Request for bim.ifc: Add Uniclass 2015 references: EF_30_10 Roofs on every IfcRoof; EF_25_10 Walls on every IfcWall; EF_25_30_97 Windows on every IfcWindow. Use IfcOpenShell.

First a look at what the model holds.

```python
import ifcopenshell

model = ifcopenshell.open("bim.ifc")
print(model.schema)
print("classifications:", [c.Name for c in model.by_type("IfcClassification")])
for ifc_class in ("IfcDoor", "IfcRoof", "IfcStair", "IfcWall", "IfcWindow"):
    print(ifc_class, len(model.by_type(ifc_class)))
```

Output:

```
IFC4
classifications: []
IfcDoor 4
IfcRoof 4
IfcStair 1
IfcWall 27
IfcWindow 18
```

```python
import ifcopenshell
import ifcopenshell.api.classification

model = ifcopenshell.open("bim.ifc")

system = ifcopenshell.api.classification.add_classification(model, classification="Uniclass 2015")

codes = {
    "IfcRoof": ("EF_30_10", "Roofs"),
    "IfcWall": ("EF_25_10", "Walls"),
    "IfcWindow": ("EF_25_30_97", "Windows"),
}
for ifc_class, (code, name) in codes.items():
    products = model.by_type(ifc_class)
    ifcopenshell.api.classification.add_reference(
        model, products=products, classification=system, identification=code, name=name
    )
    print(code, len(products))

model.write("bim_rev.ifc")
```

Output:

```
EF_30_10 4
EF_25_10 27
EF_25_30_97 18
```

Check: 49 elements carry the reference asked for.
